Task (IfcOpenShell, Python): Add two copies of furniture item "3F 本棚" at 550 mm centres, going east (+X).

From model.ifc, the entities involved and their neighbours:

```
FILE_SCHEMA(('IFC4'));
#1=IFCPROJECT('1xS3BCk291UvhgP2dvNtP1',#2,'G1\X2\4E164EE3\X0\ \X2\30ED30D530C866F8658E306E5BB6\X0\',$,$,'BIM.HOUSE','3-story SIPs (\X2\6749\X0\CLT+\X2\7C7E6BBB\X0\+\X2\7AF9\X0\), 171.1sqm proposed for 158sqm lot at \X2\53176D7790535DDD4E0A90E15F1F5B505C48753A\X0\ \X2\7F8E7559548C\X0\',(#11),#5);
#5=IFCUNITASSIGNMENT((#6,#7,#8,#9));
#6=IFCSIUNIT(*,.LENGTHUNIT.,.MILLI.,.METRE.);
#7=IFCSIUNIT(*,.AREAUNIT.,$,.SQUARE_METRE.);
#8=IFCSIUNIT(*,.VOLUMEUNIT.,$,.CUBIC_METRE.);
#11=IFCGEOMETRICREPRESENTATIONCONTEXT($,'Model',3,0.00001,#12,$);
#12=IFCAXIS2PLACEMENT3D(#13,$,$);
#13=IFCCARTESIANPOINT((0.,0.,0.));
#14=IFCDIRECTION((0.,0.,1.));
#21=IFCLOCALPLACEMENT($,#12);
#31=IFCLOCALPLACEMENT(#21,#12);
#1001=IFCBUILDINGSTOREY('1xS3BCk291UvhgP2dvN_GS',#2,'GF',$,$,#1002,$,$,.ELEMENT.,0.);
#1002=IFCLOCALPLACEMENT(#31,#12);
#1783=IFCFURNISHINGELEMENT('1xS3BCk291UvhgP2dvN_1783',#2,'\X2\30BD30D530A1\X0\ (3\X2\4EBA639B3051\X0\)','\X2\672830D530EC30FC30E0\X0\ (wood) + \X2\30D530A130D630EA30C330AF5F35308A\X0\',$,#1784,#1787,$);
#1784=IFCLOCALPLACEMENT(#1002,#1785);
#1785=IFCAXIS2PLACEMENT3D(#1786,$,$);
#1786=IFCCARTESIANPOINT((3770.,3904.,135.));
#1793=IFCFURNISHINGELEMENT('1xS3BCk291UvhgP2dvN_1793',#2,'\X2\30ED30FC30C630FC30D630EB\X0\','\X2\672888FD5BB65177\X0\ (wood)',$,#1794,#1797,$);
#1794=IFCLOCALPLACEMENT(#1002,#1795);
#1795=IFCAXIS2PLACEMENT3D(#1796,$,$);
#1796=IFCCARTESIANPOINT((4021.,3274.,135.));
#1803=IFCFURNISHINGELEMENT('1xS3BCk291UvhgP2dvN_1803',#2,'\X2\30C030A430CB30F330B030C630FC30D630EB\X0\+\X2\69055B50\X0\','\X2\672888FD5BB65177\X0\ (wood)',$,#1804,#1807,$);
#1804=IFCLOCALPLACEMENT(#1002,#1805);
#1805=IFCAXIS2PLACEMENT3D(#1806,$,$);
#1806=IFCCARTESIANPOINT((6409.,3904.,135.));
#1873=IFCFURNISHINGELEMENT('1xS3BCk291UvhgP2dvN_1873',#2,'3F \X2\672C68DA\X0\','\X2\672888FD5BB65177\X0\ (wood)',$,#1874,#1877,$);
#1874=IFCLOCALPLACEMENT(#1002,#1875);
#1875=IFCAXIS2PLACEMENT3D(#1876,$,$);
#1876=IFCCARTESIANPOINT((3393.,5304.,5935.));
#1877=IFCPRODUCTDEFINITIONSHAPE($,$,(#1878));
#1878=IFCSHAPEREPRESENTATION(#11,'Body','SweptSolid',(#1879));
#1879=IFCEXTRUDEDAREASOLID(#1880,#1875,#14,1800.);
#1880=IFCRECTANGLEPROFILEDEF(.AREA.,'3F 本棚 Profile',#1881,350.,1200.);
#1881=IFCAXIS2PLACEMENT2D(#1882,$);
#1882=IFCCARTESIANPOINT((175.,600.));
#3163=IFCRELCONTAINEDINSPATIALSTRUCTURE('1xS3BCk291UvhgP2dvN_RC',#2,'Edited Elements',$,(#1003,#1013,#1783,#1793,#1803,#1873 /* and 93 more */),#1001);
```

```python
import numpy as np
import ifcopenshell
import ifcopenshell.api.geometry
import ifcopenshell.api.root
import ifcopenshell.util.element
import ifcopenshell.util.placement
import ifcopenshell.util.unit

model = ifcopenshell.open("model.ifc")
unit_scale = ifcopenshell.util.unit.calculate_unit_scale(model)


def reuse_history(source, copy):
    """copy_class also copies each property set's owner history, people and application; keep the originals."""
    for rel in copy.IsDefinedBy:
        if rel.is_a("IfcRelDefinesByProperties") and (history := rel.RelatingPropertyDefinition.OwnerHistory):
            rel.RelatingPropertyDefinition.OwnerHistory = source.OwnerHistory
            ifcopenshell.util.element.remove_deep2(model, history)


source = model.by_guid("1xS3BCk291UvhgP2dvN_1873")
base = ifcopenshell.util.placement.get_local_placement(source.ObjectPlacement)
step = np.array([1.0, 0.0, 0.0]) * 0.55 / unit_scale

for i in range(1, 3):
    copy = ifcopenshell.api.root.copy_class(model, product=source)
    copy.Representation = ifcopenshell.util.element.copy_deep(
        model, source.Representation, exclude=["IfcGeometricRepresentationContext", "IfcRepresentationMap"]
    )
    reuse_history(source, copy)
    matrix = base.copy()
    matrix[:3, 3] += i * step
    print("added at", matrix[:3, 3].round(3) + 0.0)
    ifcopenshell.api.geometry.edit_object_placement(model, product=copy, matrix=matrix, is_si=False)

model.write("model_rev.ifc")
```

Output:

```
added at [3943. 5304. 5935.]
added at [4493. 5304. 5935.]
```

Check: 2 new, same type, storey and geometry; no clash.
